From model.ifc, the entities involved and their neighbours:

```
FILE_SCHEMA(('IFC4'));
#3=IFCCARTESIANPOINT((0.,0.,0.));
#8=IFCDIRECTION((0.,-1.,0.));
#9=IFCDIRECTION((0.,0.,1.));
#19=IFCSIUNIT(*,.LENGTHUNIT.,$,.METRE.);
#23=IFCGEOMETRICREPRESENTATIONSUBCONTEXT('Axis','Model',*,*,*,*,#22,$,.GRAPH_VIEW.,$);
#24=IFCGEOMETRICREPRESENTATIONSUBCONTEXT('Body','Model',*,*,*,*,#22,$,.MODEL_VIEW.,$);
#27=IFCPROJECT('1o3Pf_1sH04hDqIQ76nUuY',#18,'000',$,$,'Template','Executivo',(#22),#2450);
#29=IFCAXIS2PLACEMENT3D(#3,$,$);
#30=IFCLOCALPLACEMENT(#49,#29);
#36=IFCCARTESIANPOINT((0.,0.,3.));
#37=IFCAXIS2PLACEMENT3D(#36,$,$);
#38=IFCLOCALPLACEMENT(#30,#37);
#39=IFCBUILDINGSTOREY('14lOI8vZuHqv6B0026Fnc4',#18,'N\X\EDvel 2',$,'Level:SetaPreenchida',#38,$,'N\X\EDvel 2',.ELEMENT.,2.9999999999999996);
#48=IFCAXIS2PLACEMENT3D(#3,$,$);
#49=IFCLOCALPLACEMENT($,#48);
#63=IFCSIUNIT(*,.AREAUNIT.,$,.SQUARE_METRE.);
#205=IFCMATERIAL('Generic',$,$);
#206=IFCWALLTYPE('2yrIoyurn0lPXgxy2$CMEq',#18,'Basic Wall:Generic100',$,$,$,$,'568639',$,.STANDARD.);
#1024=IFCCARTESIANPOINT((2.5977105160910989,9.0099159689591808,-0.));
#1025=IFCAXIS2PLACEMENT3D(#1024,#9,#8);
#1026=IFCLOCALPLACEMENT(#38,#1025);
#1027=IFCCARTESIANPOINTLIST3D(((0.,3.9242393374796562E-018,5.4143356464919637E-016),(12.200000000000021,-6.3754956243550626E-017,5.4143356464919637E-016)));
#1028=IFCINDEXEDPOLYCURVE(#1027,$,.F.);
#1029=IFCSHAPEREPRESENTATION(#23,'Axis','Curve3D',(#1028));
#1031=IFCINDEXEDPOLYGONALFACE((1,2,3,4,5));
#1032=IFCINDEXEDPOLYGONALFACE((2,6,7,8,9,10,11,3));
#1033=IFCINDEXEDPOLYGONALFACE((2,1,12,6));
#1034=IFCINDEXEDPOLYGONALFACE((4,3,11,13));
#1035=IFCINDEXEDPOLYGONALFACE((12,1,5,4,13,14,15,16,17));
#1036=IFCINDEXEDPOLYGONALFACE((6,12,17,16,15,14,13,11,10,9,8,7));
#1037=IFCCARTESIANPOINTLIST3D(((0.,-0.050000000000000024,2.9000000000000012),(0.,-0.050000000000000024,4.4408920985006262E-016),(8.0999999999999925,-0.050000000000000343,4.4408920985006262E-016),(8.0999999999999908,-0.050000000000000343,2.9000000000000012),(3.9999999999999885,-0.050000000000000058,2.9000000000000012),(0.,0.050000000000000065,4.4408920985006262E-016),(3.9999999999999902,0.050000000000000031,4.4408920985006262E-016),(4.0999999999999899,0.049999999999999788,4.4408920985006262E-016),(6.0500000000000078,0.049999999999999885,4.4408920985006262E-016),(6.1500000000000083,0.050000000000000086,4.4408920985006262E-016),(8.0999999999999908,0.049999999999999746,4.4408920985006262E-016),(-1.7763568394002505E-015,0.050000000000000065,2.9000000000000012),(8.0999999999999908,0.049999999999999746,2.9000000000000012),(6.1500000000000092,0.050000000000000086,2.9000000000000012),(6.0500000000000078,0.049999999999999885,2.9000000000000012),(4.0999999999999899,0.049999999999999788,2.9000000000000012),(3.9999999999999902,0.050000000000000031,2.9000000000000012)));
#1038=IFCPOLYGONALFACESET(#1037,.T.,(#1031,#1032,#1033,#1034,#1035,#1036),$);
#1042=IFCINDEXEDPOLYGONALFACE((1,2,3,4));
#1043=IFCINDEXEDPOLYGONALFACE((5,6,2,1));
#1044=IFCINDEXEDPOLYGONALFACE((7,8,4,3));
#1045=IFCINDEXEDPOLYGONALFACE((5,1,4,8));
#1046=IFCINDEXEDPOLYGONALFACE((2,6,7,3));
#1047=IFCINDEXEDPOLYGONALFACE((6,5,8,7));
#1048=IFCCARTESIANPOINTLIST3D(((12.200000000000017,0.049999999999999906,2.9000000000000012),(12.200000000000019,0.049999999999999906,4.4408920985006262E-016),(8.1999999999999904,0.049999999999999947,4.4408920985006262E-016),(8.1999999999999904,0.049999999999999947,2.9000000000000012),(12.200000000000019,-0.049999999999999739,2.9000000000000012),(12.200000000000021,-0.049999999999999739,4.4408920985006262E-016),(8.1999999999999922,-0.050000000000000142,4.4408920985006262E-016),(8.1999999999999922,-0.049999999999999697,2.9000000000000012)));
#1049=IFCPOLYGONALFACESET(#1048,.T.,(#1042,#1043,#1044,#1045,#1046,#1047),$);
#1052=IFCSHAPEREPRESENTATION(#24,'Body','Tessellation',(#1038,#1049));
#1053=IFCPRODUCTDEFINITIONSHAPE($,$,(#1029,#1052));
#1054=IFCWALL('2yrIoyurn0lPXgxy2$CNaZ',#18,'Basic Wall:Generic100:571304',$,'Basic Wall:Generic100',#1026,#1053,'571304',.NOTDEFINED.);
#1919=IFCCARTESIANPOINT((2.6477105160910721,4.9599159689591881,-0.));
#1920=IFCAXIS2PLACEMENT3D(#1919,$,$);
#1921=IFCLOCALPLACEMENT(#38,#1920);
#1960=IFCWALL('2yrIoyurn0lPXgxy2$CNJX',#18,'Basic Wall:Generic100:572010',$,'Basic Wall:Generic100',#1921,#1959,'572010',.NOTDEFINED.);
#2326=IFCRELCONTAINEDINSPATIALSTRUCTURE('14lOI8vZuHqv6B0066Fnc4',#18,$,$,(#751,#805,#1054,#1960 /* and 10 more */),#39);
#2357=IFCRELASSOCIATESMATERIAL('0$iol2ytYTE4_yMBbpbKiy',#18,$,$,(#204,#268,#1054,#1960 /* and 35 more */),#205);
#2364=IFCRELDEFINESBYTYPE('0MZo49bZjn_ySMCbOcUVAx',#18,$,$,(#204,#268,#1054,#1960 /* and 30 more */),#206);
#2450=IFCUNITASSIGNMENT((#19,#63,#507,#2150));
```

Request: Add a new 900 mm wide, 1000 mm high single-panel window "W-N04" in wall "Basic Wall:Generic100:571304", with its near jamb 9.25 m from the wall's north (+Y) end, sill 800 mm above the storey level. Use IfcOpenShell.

```python
import numpy as np
import ifcopenshell
import ifcopenshell.api.feature
import ifcopenshell.api.geometry
import ifcopenshell.api.root
import ifcopenshell.api.spatial
import ifcopenshell.geom
import ifcopenshell.util.element
import ifcopenshell.util.placement
import ifcopenshell.util.representation
import ifcopenshell.util.shape
import ifcopenshell.util.unit

model = ifcopenshell.open("model.ifc")
unit_scale = ifcopenshell.util.unit.calculate_unit_scale(model)
settings = ifcopenshell.geom.settings()


def volume(element):
    """Net volume in cubic metres, openings subtracted."""
    shape = ifcopenshell.geom.create_shape(settings, element)
    return ifcopenshell.util.shape.get_volume(shape.geometry)


wall = model.by_guid("2yrIoyurn0lPXgxy2$CNaZ")
storey = ifcopenshell.util.element.get_container(wall, ifc_class="IfcBuildingStorey")
context = ifcopenshell.util.representation.get_context(model, "Model", "Body", "MODEL_VIEW")
before = volume(wall)

width, height, from_end, sill = 0.9, 1, 9.25, 0.8  # metres

# The wall runs along its own X axis, and the end named is its -X end.
wall_shape = ifcopenshell.geom.create_shape(settings, wall)
x, y, z = ifcopenshell.util.shape.get_vertices(wall_shape.geometry).T
start = x.min() + from_end
face, thickness = float(y.min()), float(y.max() - y.min())
wall_matrix = ifcopenshell.util.placement.get_local_placement(wall.ObjectPlacement)
level = ifcopenshell.util.placement.get_local_placement(storey.ObjectPlacement)[2, 3]


def in_wall(x, y):
    """Placement at x, y metres in the wall's axes, at sill height."""
    matrix = wall_matrix.copy()
    matrix[:, 3] = wall_matrix @ np.array([x / unit_scale, y / unit_scale, 0.0, 1.0])
    matrix[2, 3] = level + sill / unit_scale
    return matrix


# Opening: a box that overshoots both wall faces by 50 mm.
opening = ifcopenshell.api.root.create_entity(model, ifc_class="IfcOpeningElement", predefined_type="OPENING")
box = ifcopenshell.api.geometry.add_wall_representation(
    model, context=context, length=width, height=height, thickness=thickness + 0.1
)
ifcopenshell.api.geometry.assign_representation(model, product=opening, representation=box)
ifcopenshell.api.geometry.edit_object_placement(model, product=opening, matrix=in_wall(start, face - 0.05), is_si=False)
ifcopenshell.api.feature.add_feature(model, feature=opening, element=wall)

window = ifcopenshell.api.root.create_entity(model, ifc_class="IfcWindow", name="W-N04", predefined_type="WINDOW")
window.OverallWidth, window.OverallHeight = width / unit_scale, height / unit_scale
window.PartitioningType = "SINGLE_PANEL"
body = ifcopenshell.api.geometry.add_window_representation(
    model,
    context=context,
    overall_width=window.OverallWidth,
    overall_height=window.OverallHeight,
    partition_type="SINGLE_PANEL",
)
ifcopenshell.api.geometry.assign_representation(model, product=window, representation=body)
ifcopenshell.api.spatial.assign_container(model, products=[window], relating_structure=storey)
ifcopenshell.api.feature.add_filling(model, opening=opening, element=window)

# Centre the window in the wall's thickness.
ifcopenshell.api.geometry.edit_object_placement(model, product=window, matrix=in_wall(start, face), is_si=False)
window_shape = ifcopenshell.geom.create_shape(settings, window)
depth = ifcopenshell.util.shape.get_vertices(window_shape.geometry)[:, 1]
offset = face + thickness / 2 - (depth.min() + depth.max()) / 2
ifcopenshell.api.geometry.edit_object_placement(model, product=window, matrix=in_wall(start, offset), is_si=False)

after = volume(wall)

print(f"wall volume {before:.3f} -> {after:.3f} m3")

model.write("model_rev.ifc")
```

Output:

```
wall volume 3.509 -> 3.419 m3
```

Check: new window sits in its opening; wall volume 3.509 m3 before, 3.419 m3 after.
